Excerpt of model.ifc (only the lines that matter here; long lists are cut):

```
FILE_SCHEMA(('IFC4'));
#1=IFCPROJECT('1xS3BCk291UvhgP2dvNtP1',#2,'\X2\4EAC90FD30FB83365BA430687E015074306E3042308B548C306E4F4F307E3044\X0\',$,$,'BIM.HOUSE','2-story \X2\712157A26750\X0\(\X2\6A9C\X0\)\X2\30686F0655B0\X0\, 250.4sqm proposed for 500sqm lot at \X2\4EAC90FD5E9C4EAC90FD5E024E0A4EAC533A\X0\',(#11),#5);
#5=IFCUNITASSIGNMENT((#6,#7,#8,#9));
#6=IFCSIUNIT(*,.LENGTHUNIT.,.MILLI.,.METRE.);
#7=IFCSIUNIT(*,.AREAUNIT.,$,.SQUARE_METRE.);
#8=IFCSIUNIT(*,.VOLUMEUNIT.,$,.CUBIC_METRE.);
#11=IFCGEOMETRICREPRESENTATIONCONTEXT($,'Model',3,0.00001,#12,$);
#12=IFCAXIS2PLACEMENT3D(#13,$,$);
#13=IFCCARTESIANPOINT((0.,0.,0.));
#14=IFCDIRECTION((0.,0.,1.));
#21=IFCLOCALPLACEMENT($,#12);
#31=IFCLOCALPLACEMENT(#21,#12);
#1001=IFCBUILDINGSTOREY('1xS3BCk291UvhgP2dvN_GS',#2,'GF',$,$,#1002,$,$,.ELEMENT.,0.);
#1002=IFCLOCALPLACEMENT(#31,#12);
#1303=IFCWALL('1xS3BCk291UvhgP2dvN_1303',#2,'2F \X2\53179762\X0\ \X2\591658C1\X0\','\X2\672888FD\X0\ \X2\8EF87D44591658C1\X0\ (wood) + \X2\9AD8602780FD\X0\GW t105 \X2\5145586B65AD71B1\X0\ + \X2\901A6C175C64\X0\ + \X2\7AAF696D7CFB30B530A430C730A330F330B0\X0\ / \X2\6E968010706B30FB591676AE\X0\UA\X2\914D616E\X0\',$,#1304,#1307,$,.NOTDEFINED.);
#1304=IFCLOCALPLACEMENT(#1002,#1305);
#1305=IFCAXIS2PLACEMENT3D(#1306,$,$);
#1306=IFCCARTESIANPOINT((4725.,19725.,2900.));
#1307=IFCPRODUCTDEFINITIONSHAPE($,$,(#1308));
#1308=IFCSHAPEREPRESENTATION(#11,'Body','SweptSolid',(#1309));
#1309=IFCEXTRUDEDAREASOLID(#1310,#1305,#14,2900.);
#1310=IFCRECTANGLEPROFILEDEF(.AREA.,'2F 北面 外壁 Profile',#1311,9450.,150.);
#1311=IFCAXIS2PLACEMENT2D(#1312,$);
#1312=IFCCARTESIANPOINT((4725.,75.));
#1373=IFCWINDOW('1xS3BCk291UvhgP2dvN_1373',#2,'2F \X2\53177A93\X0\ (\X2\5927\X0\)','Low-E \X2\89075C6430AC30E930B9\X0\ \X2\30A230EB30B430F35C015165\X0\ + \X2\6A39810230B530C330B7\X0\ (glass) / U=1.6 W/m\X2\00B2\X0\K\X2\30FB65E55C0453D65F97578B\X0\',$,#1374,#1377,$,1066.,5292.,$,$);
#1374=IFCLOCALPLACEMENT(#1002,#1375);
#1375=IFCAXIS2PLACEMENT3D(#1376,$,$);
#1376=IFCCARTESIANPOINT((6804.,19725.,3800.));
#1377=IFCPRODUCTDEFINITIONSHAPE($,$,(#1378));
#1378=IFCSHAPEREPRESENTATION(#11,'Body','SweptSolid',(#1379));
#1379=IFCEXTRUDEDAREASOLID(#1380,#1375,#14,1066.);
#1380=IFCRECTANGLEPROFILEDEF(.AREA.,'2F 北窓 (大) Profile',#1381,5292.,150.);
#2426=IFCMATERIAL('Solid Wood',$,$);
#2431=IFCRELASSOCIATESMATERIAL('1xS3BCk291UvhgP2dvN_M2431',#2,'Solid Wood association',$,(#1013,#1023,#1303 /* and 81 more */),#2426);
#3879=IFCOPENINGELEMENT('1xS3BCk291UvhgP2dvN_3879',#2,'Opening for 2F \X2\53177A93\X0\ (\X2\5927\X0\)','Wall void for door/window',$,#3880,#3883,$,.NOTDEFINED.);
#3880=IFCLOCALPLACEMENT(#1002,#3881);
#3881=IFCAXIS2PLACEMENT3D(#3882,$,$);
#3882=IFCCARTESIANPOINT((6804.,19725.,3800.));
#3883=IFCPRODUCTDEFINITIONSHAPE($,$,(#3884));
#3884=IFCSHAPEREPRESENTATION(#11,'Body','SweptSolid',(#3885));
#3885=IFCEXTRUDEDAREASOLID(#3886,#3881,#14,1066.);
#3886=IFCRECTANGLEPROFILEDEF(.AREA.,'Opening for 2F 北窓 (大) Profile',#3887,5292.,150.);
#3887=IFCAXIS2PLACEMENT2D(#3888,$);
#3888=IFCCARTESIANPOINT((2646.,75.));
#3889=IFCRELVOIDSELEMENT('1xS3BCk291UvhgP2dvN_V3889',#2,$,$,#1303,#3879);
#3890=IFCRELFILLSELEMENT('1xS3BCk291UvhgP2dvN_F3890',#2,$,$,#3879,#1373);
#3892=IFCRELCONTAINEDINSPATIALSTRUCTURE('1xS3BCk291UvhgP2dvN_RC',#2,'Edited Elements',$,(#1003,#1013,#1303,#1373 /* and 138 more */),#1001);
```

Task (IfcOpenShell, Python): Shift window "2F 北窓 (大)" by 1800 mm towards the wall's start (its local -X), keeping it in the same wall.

```python
import ifcopenshell
import ifcopenshell.api.geometry
import ifcopenshell.util.placement
import ifcopenshell.util.unit

model = ifcopenshell.open("model.ifc")
unit_scale = ifcopenshell.util.unit.calculate_unit_scale(model)

window = model.by_guid("1xS3BCk291UvhgP2dvN_1373")
opening = window.FillsVoids[0].RelatingOpeningElement
wall = opening.VoidsElements[0].RelatingBuildingElement

wall_matrix = ifcopenshell.util.placement.get_local_placement(wall.ObjectPlacement)
shift = wall_matrix[:3, 0] * -1.8 / unit_scale
before = ifcopenshell.util.placement.get_local_placement(window.ObjectPlacement)[:3, 3].copy()

# The window is not placed relative to its opening, so move both.
for product in (opening, window):
    matrix = ifcopenshell.util.placement.get_local_placement(product.ObjectPlacement)
    matrix[:3, 3] += shift
    ifcopenshell.api.geometry.edit_object_placement(model, product=product, matrix=matrix, is_si=False)

after = ifcopenshell.util.placement.get_local_placement(window.ObjectPlacement)[:3, 3]
print("window moved by", (after - before).round(3) + 0.0)

model.write("model-out.ifc")
```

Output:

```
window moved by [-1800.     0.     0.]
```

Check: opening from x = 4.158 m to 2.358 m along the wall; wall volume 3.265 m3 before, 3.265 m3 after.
